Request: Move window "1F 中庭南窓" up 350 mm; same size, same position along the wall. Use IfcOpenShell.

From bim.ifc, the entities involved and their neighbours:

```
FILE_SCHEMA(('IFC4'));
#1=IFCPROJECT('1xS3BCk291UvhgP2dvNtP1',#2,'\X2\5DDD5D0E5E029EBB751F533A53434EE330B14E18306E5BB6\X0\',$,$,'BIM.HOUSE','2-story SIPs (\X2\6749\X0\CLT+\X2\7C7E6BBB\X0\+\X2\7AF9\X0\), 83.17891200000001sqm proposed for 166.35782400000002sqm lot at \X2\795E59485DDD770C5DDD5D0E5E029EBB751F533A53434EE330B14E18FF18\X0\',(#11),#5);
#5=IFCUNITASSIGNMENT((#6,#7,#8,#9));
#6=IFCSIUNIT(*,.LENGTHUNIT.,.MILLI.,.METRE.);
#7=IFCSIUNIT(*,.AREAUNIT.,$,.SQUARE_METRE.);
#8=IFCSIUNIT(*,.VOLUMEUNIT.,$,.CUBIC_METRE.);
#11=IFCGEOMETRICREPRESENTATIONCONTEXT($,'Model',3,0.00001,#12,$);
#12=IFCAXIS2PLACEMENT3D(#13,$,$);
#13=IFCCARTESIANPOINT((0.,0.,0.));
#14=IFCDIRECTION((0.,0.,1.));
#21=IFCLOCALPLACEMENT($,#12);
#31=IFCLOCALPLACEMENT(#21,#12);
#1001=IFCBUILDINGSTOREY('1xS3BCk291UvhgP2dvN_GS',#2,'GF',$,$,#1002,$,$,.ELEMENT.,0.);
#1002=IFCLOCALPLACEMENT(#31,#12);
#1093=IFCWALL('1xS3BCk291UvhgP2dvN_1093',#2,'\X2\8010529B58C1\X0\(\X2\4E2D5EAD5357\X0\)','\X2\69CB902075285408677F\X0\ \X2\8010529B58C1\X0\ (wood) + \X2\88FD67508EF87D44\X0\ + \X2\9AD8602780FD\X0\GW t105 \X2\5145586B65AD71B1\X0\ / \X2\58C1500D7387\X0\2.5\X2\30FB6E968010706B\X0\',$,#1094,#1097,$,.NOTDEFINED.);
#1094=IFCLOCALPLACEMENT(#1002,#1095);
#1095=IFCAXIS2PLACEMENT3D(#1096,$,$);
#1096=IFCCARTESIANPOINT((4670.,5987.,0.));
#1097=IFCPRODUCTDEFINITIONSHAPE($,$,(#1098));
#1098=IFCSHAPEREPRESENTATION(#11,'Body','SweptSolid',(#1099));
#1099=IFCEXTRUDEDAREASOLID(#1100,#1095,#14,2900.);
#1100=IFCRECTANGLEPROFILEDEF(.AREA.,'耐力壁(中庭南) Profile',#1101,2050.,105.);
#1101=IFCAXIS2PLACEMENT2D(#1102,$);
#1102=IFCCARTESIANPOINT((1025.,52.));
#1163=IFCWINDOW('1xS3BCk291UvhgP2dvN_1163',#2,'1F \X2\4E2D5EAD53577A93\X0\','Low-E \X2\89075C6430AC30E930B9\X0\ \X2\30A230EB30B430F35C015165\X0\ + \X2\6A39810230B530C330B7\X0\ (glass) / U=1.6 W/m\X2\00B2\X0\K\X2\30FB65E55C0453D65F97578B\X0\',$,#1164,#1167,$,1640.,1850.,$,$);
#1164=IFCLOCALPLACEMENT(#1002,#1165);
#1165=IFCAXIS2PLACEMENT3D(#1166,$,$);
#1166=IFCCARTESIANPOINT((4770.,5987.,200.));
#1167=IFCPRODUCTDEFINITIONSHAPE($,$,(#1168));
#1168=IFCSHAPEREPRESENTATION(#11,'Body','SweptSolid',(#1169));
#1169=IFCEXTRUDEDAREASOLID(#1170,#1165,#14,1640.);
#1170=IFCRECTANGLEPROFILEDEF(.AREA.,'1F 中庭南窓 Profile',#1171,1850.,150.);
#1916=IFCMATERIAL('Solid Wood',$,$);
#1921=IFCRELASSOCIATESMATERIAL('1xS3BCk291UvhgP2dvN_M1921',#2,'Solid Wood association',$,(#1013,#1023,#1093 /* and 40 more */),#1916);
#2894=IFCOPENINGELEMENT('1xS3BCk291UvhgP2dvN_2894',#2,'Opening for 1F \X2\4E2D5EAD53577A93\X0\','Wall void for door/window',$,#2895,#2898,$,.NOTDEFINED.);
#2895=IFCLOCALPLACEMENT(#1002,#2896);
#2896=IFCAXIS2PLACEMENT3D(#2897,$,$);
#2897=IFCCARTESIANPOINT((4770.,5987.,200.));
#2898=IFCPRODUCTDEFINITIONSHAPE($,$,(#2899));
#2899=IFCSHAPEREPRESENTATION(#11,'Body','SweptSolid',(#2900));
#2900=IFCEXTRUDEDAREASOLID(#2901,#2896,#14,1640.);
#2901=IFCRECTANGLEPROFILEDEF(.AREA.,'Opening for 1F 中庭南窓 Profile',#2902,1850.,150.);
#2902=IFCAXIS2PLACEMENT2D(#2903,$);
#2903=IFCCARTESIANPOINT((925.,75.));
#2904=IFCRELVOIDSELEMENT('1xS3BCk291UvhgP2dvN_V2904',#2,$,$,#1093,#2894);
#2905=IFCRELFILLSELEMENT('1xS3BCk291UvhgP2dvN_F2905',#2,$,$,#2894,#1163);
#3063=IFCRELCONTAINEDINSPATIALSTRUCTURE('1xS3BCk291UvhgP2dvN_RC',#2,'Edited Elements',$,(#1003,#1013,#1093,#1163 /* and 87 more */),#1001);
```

```python
import numpy as np
import ifcopenshell
import ifcopenshell.api.geometry
import ifcopenshell.util.placement
import ifcopenshell.util.unit

model = ifcopenshell.open("bim.ifc")
unit_scale = ifcopenshell.util.unit.calculate_unit_scale(model)

window = model.by_guid("1xS3BCk291UvhgP2dvN_1163")
opening = window.FillsVoids[0].RelatingOpeningElement
dz = 350.0

shift = np.array([0.0, 0.0, dz])
# The window is not placed relative to its opening, so move both.
for product in (opening, window):
    matrix = ifcopenshell.util.placement.get_local_placement(product.ObjectPlacement)
    matrix[:3, 3] += shift
    ifcopenshell.api.geometry.edit_object_placement(model, product=product, matrix=matrix, is_si=False)

print(f"moved by {dz * unit_scale:+.3f} m")

model.write("bim_rev.ifc")
```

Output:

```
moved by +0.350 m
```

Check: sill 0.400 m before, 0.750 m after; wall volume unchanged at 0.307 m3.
